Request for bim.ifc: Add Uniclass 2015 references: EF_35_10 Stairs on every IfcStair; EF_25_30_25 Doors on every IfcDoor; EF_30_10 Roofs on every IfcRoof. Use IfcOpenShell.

First a look at what the model holds.

```python
import ifcopenshell

model = ifcopenshell.open("bim.ifc")
print(model.schema)
print("classifications:", [c.Name for c in model.by_type("IfcClassification")])
for ifc_class in ("IfcDoor", "IfcRoof", "IfcStair", "IfcWall", "IfcWindow"):
    print(ifc_class, len(model.by_type(ifc_class)))
```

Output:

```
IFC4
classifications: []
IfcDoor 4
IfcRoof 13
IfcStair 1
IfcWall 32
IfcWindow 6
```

```python
import ifcopenshell
import ifcopenshell.api.classification

model = ifcopenshell.open("bim.ifc")

system = ifcopenshell.api.classification.add_classification(model, classification="Uniclass 2015")

codes = {
    "IfcStair": ("EF_35_10", "Stairs"),
    "IfcDoor": ("EF_25_30_25", "Doors"),
    "IfcRoof": ("EF_30_10", "Roofs"),
}
for ifc_class, (code, name) in codes.items():
    products = model.by_type(ifc_class)
    ifcopenshell.api.classification.add_reference(
        model, products=products, classification=system, identification=code, name=name
    )
    print(code, len(products))

model.write("bim-out.ifc")
```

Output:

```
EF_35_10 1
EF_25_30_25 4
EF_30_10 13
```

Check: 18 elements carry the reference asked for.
